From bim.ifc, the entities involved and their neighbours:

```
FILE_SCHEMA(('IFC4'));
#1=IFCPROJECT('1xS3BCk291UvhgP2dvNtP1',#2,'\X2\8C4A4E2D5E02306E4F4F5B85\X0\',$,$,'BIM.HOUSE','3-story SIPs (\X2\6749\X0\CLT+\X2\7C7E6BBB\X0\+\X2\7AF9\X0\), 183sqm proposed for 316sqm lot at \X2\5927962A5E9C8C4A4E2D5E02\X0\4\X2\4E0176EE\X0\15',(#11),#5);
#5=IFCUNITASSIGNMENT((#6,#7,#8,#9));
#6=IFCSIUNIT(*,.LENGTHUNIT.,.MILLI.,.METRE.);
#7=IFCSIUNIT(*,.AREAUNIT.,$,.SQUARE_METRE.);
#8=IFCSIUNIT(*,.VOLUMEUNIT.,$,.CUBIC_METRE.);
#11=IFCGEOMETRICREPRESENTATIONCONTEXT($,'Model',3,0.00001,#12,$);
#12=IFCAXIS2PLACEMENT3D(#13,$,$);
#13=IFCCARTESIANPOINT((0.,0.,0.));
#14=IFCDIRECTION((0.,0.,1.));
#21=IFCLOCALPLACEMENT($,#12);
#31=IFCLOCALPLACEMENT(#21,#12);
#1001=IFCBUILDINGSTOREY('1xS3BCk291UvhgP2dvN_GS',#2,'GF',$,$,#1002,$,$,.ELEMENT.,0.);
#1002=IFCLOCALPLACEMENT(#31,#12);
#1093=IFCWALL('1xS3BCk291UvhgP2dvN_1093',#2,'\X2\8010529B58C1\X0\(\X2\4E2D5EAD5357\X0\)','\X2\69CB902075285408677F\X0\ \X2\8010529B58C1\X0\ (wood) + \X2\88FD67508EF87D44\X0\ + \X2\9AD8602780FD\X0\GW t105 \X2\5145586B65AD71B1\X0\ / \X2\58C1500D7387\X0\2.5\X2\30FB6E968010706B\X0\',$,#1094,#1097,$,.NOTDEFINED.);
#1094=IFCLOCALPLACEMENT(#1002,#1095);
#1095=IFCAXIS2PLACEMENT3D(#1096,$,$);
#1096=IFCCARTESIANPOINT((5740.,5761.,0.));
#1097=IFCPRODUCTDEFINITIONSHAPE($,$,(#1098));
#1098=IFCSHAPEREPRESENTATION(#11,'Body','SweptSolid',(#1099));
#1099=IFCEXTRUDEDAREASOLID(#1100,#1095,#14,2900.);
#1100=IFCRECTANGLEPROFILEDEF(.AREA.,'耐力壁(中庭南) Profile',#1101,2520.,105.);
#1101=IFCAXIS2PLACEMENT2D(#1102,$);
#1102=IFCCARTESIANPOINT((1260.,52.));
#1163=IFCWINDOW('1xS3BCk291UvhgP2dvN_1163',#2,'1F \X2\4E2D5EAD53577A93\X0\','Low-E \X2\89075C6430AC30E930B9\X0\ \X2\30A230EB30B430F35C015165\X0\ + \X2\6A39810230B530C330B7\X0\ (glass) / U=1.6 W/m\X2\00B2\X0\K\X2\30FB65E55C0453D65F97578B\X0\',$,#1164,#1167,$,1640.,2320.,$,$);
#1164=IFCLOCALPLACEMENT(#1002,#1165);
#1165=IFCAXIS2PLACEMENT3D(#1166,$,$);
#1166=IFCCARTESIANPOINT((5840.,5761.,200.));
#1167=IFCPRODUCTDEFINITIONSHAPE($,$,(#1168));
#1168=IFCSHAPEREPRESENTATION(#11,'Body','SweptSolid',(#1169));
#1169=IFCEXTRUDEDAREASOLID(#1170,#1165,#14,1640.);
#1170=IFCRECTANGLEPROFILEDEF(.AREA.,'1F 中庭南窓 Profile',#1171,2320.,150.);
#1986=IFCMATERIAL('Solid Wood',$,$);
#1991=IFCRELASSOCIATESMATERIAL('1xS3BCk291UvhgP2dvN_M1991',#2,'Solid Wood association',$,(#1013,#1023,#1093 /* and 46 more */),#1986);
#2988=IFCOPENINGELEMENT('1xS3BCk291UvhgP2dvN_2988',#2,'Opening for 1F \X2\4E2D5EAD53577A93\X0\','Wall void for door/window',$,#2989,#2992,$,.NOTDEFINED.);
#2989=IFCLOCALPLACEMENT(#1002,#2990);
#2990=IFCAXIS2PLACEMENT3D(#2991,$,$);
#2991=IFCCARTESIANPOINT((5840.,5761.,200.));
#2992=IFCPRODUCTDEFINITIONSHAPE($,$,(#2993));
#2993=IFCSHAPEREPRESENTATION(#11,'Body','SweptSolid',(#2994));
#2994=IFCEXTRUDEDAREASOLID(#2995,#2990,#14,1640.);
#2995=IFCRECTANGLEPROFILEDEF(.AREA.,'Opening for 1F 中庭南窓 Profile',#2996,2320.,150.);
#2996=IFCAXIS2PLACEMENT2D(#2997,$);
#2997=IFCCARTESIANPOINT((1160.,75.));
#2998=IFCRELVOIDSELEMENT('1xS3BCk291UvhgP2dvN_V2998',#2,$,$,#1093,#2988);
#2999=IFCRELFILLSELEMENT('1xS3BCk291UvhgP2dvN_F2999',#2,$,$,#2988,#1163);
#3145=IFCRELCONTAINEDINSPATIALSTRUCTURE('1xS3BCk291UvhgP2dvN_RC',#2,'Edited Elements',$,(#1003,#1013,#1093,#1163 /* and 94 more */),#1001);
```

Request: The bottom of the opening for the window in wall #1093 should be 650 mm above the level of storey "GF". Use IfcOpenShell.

```python
import numpy as np
import ifcopenshell
import ifcopenshell.api.geometry
import ifcopenshell.geom
import ifcopenshell.util.element
import ifcopenshell.util.placement
import ifcopenshell.util.shape
import ifcopenshell.util.unit

model = ifcopenshell.open("bim.ifc")
unit_scale = ifcopenshell.util.unit.calculate_unit_scale(model)

window = model.by_guid("1xS3BCk291UvhgP2dvN_1163")
opening = window.FillsVoids[0].RelatingOpeningElement
storey = ifcopenshell.util.element.get_container(window, ifc_class="IfcBuildingStorey")
level = ifcopenshell.util.placement.get_local_placement(storey.ObjectPlacement)[2, 3]

# The opening's origin need not be at the sill, so measure its lowest point.
shape = ifcopenshell.geom.create_shape(ifcopenshell.geom.settings(), opening)
bottom = ifcopenshell.util.shape.get_shape_bottom_elevation(shape, shape.geometry) / unit_scale
dz = level + 650.0 - bottom

shift = np.array([0.0, 0.0, dz])
# The window is not placed relative to its opening, so move both.
for product in (opening, window):
    matrix = ifcopenshell.util.placement.get_local_placement(product.ObjectPlacement)
    matrix[:3, 3] += shift
    ifcopenshell.api.geometry.edit_object_placement(model, product=product, matrix=matrix, is_si=False)

print(f"moved by {dz * unit_scale:+.3f} m")

model.write("bim_rev.ifc")
```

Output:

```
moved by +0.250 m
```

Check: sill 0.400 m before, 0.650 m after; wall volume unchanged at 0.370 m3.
